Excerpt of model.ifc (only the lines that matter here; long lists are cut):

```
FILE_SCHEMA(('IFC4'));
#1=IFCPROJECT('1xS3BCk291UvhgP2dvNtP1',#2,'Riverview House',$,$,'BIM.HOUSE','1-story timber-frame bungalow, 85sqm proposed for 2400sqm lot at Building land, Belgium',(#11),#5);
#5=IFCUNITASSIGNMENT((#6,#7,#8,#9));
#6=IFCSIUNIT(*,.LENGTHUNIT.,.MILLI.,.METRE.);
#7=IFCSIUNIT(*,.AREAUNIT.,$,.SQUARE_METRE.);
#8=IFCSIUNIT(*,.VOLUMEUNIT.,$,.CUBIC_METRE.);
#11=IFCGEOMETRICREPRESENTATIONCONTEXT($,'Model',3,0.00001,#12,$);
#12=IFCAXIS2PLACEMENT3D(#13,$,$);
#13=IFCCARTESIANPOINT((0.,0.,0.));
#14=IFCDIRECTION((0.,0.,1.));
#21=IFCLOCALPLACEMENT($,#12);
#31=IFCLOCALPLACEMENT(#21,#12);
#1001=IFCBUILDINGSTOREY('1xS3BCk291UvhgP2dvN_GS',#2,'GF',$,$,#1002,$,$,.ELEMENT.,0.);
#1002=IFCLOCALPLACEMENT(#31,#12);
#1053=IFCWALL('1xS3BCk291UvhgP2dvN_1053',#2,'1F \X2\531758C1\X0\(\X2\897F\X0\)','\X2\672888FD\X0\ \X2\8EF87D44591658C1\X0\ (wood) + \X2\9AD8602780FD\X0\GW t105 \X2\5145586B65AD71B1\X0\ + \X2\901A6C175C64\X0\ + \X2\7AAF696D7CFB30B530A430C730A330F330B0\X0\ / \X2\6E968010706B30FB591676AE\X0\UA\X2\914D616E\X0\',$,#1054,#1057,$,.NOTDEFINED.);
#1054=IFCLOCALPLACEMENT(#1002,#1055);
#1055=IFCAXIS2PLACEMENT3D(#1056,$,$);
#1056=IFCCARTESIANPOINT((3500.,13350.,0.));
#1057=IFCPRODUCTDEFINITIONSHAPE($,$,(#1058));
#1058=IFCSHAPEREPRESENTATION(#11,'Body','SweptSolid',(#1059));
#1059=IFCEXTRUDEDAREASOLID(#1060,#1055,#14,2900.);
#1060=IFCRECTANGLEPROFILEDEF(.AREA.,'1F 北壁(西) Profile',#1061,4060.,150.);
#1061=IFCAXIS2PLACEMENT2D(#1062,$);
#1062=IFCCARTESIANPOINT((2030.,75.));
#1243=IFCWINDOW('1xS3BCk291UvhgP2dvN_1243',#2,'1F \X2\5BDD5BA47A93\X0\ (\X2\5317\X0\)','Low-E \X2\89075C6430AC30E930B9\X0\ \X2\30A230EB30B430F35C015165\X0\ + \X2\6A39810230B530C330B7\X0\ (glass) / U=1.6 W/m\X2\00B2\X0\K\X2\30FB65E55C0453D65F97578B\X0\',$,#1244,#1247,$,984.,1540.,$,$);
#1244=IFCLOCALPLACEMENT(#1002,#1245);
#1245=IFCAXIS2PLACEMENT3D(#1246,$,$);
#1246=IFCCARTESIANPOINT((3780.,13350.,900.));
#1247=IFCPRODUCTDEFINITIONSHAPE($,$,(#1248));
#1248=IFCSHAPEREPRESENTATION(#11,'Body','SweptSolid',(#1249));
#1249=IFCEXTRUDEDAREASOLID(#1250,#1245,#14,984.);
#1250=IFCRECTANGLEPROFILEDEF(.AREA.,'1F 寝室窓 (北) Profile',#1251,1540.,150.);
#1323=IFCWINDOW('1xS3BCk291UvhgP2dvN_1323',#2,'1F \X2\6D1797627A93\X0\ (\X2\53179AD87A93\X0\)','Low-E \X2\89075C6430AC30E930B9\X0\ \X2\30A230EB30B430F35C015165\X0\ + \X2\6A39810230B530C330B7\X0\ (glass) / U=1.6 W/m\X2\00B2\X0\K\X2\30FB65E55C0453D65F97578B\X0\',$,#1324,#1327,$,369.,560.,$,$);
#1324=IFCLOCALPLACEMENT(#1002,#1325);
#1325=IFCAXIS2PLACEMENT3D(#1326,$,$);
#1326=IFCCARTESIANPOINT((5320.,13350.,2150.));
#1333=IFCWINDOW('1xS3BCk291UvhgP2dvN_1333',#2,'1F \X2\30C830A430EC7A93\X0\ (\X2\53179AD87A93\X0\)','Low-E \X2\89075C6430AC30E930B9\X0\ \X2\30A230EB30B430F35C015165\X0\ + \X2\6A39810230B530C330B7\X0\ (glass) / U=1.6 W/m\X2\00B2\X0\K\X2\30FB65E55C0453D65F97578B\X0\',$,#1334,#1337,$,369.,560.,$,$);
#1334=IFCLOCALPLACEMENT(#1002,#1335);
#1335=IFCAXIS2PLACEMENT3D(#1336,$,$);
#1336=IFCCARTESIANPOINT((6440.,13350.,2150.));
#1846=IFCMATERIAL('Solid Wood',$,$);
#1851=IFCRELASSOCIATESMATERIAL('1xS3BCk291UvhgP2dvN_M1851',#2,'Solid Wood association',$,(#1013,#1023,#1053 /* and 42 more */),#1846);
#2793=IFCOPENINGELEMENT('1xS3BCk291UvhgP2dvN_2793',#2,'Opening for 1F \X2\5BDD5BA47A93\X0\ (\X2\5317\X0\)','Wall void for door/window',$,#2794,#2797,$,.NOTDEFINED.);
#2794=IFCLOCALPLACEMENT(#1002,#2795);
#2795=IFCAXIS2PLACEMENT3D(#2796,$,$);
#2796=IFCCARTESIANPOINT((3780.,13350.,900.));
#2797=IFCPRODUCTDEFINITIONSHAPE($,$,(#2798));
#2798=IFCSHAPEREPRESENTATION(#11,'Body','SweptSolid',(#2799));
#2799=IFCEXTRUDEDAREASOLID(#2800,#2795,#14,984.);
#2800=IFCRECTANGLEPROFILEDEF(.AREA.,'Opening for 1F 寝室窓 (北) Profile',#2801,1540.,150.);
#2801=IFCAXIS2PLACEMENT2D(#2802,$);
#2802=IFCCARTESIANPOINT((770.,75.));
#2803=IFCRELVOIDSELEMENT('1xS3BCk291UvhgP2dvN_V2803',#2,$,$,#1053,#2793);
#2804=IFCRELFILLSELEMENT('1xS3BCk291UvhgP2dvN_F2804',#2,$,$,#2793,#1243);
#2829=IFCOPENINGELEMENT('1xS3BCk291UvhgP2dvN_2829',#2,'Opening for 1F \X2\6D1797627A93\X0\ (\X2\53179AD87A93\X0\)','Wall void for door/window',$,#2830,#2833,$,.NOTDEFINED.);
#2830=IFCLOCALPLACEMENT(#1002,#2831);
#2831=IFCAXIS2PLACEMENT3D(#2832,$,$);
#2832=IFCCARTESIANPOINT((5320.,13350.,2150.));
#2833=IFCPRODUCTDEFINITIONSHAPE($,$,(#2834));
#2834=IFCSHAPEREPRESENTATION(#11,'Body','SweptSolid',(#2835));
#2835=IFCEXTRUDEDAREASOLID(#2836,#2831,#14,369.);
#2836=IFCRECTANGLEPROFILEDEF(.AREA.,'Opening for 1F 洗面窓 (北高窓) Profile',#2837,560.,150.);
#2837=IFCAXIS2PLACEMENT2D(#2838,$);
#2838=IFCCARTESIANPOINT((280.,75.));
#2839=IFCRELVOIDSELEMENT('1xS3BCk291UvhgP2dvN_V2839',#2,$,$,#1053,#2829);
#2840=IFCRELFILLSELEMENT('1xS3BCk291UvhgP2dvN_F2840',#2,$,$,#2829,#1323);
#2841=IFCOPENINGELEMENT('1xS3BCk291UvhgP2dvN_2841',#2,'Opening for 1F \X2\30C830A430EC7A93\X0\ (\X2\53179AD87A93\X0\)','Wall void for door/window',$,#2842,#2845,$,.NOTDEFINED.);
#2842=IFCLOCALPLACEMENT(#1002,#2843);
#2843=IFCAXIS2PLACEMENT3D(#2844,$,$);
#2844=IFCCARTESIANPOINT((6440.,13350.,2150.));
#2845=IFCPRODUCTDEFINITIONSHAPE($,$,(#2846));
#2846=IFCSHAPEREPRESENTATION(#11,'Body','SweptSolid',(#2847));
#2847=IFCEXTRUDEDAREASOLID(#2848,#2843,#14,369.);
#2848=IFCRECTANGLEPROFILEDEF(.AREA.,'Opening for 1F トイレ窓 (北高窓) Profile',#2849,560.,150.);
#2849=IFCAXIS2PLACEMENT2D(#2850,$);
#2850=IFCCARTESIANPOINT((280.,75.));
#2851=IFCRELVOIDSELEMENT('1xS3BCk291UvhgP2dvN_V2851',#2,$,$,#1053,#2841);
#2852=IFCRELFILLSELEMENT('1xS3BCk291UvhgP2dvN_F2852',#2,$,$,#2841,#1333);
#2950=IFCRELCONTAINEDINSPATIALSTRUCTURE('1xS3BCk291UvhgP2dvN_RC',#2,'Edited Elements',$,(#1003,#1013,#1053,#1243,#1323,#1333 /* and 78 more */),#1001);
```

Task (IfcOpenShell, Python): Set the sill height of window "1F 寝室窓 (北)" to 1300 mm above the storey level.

```python
import numpy as np
import ifcopenshell
import ifcopenshell.api.geometry
import ifcopenshell.geom
import ifcopenshell.util.element
import ifcopenshell.util.placement
import ifcopenshell.util.shape
import ifcopenshell.util.unit

model = ifcopenshell.open("model.ifc")
unit_scale = ifcopenshell.util.unit.calculate_unit_scale(model)

window = model.by_guid("1xS3BCk291UvhgP2dvN_1243")
opening = window.FillsVoids[0].RelatingOpeningElement
storey = ifcopenshell.util.element.get_container(window, ifc_class="IfcBuildingStorey")
level = ifcopenshell.util.placement.get_local_placement(storey.ObjectPlacement)[2, 3]

# The opening's origin need not be at the sill, so measure its lowest point.
shape = ifcopenshell.geom.create_shape(ifcopenshell.geom.settings(), opening)
bottom = ifcopenshell.util.shape.get_shape_bottom_elevation(shape, shape.geometry) / unit_scale
dz = level + 1.3 / unit_scale - bottom

shift = np.array([0.0, 0.0, dz])
# The window is not placed relative to its opening, so move both.
for product in (opening, window):
    matrix = ifcopenshell.util.placement.get_local_placement(product.ObjectPlacement)
    matrix[:3, 3] += shift
    ifcopenshell.api.geometry.edit_object_placement(model, product=product, matrix=matrix, is_si=False)

print(f"moved by {dz * unit_scale:+.3f} m")

model.write("model-out.ifc")
```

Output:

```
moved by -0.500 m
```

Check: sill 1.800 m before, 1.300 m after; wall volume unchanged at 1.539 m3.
